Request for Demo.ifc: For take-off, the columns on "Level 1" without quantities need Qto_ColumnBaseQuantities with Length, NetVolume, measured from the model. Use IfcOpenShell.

First a look at what the model holds.

```python
import ifcopenshell
import ifcopenshell.util.element
import ifcopenshell.util.unit

model = ifcopenshell.open("Demo.ifc")
print(model.schema)
for unit_type in ("LENGTHUNIT", "AREAUNIT", "VOLUMEUNIT"):
    print(unit_type, ifcopenshell.util.unit.calculate_unit_scale(model, unit_type))
storey = next(s for s in model.by_type("IfcBuildingStorey") if s.Name == "Level 1")
columns = [e for e in ifcopenshell.util.element.get_decomposition(storey) if e.is_a("IfcColumn")]
for e in sorted(columns, key=lambda e: e.id()):
    print(e.id(), e.is_a(), e.Name, list(ifcopenshell.util.element.get_psets(e, qtos_only=True)), sep=" | ")
```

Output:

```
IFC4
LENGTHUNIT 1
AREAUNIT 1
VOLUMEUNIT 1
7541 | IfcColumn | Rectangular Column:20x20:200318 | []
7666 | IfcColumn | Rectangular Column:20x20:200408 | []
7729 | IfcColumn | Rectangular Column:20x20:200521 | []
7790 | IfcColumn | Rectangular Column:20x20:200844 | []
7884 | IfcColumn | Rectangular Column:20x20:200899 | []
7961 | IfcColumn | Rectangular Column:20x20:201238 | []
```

```python
import ifcopenshell
import ifcopenshell.api.pset
import ifcopenshell.geom
import ifcopenshell.util.element
import ifcopenshell.util.shape
import ifcopenshell.util.unit

model = ifcopenshell.open("Demo.ifc")
unit_scale = ifcopenshell.util.unit.calculate_unit_scale(model)
volume_scale = ifcopenshell.util.unit.calculate_unit_scale(model, "VOLUMEUNIT")
settings = ifcopenshell.geom.settings()

storey = next(s for s in model.by_type("IfcBuildingStorey") if s.Name == "Level 1")
columns = [e for e in ifcopenshell.util.element.get_decomposition(storey) if e.is_a("IfcColumn")]

for e in sorted(columns, key=lambda e: e.id()):
    if ifcopenshell.util.element.get_psets(e, qtos_only=True, should_inherit=False):
        continue
    # Geometry comes back in metres, in the element's own axes.
    shape = ifcopenshell.geom.create_shape(settings, e)
    values = {
        "Length": ifcopenshell.util.shape.get_z(shape.geometry) / unit_scale,
        "NetVolume": ifcopenshell.util.shape.get_volume(shape.geometry) / volume_scale,
    }
    qto = ifcopenshell.api.pset.add_qto(model, product=e, name="Qto_ColumnBaseQuantities")
    ifcopenshell.api.pset.edit_qto(model, qto=qto, properties=values)
    print(e.id(), {k: round(v, 3) for k, v in values.items()})

model.write("Demo_updated.ifc")
```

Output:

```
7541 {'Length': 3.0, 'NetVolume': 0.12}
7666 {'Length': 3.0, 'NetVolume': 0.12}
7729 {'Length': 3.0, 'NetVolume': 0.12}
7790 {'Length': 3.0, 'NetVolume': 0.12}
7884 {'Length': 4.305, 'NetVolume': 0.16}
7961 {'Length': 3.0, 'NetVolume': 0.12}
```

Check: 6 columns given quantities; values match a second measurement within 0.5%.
